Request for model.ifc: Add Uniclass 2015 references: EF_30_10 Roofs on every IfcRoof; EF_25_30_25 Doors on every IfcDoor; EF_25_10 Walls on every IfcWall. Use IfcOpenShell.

First a look at what the model holds.

```python
import ifcopenshell

model = ifcopenshell.open("model.ifc")
print(model.schema)
print("classifications:", [c.Name for c in model.by_type("IfcClassification")])
for ifc_class in ("IfcDoor", "IfcRoof", "IfcStair", "IfcWall", "IfcWindow"):
    print(ifc_class, len(model.by_type(ifc_class)))
```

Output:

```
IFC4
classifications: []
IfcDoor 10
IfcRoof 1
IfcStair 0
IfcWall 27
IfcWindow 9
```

```python
import ifcopenshell
import ifcopenshell.api.classification

model = ifcopenshell.open("model.ifc")

system = ifcopenshell.api.classification.add_classification(model, classification="Uniclass 2015")

codes = {
    "IfcRoof": ("EF_30_10", "Roofs"),
    "IfcDoor": ("EF_25_30_25", "Doors"),
    "IfcWall": ("EF_25_10", "Walls"),
}
for ifc_class, (code, name) in codes.items():
    products = model.by_type(ifc_class)
    ifcopenshell.api.classification.add_reference(
        model, products=products, classification=system, identification=code, name=name
    )
    print(code, len(products))

model.write("model_rev.ifc")
```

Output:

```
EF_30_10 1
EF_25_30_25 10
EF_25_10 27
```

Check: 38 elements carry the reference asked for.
